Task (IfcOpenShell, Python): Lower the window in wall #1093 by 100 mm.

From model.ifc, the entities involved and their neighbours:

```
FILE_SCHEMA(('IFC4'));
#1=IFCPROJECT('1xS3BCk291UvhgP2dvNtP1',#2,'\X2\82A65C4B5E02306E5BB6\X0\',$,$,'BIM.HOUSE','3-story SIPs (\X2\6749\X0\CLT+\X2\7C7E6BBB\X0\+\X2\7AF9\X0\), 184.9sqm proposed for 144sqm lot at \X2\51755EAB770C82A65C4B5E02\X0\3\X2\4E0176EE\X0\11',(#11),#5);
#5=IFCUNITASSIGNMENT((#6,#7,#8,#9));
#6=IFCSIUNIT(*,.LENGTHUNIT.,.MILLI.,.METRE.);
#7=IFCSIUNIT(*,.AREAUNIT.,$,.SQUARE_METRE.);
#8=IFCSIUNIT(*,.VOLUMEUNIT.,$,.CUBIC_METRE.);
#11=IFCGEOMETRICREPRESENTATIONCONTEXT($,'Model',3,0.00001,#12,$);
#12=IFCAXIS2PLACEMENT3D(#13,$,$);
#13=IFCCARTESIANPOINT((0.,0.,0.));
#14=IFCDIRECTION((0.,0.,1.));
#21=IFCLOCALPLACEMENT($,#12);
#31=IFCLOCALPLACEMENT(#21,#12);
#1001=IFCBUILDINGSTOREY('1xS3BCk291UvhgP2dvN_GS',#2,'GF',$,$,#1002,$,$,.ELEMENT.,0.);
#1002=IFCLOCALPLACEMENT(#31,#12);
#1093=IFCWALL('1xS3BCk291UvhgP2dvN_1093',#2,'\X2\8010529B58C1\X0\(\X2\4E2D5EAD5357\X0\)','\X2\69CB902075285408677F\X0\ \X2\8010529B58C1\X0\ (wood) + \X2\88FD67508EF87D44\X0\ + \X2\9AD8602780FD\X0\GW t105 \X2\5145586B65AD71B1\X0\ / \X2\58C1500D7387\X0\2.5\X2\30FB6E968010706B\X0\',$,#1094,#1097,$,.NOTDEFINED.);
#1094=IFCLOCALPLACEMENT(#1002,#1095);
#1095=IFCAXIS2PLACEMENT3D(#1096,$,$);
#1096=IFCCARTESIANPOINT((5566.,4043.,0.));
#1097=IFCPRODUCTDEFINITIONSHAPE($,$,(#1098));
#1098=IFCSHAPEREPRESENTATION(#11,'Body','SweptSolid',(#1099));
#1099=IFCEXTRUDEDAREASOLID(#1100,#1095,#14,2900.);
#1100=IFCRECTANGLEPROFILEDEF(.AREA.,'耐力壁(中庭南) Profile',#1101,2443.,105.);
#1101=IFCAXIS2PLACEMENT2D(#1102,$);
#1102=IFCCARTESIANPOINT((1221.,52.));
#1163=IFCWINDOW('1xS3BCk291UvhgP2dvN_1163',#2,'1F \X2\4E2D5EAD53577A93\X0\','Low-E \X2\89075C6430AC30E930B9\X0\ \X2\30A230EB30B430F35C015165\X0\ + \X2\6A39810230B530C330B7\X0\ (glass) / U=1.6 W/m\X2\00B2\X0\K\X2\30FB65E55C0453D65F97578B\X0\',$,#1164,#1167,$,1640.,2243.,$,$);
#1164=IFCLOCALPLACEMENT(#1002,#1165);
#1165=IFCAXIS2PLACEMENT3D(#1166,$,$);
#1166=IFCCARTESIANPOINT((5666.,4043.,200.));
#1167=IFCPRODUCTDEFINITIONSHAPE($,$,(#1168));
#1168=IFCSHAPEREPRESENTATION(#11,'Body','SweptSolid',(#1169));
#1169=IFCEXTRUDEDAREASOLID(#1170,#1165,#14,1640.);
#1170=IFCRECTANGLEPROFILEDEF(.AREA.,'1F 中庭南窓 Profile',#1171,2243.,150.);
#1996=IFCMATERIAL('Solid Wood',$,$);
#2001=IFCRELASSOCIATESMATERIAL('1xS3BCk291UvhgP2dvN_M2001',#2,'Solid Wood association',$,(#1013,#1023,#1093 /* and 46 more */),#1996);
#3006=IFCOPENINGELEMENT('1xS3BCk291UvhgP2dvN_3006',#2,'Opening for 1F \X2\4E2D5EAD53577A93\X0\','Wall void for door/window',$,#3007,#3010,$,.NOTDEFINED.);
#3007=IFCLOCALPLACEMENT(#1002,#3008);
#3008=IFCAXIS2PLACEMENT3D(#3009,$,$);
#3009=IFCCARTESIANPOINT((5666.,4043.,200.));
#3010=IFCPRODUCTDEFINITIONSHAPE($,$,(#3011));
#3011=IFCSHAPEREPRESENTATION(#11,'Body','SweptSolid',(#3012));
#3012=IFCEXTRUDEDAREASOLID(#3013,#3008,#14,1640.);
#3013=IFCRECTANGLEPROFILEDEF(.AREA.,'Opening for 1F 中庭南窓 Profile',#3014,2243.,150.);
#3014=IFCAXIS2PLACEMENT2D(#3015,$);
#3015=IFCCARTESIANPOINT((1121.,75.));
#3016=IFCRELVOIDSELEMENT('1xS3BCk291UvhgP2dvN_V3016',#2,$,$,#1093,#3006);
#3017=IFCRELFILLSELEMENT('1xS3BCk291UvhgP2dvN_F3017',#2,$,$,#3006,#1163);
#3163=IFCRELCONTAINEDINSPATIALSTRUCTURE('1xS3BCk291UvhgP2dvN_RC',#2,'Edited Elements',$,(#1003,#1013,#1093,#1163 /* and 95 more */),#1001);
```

```python
import numpy as np
import ifcopenshell
import ifcopenshell.api.geometry
import ifcopenshell.util.placement
import ifcopenshell.util.unit

model = ifcopenshell.open("model.ifc")
unit_scale = ifcopenshell.util.unit.calculate_unit_scale(model)

window = model.by_guid("1xS3BCk291UvhgP2dvN_1163")
opening = window.FillsVoids[0].RelatingOpeningElement
dz = -0.1 / unit_scale

shift = np.array([0.0, 0.0, dz])
# The window is not placed relative to its opening, so move both.
for product in (opening, window):
    matrix = ifcopenshell.util.placement.get_local_placement(product.ObjectPlacement)
    matrix[:3, 3] += shift
    ifcopenshell.api.geometry.edit_object_placement(model, product=product, matrix=matrix, is_si=False)

print(f"moved by {dz * unit_scale:+.3f} m")

model.write("model-out.ifc")
```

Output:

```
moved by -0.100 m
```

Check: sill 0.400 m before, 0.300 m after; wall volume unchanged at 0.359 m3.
